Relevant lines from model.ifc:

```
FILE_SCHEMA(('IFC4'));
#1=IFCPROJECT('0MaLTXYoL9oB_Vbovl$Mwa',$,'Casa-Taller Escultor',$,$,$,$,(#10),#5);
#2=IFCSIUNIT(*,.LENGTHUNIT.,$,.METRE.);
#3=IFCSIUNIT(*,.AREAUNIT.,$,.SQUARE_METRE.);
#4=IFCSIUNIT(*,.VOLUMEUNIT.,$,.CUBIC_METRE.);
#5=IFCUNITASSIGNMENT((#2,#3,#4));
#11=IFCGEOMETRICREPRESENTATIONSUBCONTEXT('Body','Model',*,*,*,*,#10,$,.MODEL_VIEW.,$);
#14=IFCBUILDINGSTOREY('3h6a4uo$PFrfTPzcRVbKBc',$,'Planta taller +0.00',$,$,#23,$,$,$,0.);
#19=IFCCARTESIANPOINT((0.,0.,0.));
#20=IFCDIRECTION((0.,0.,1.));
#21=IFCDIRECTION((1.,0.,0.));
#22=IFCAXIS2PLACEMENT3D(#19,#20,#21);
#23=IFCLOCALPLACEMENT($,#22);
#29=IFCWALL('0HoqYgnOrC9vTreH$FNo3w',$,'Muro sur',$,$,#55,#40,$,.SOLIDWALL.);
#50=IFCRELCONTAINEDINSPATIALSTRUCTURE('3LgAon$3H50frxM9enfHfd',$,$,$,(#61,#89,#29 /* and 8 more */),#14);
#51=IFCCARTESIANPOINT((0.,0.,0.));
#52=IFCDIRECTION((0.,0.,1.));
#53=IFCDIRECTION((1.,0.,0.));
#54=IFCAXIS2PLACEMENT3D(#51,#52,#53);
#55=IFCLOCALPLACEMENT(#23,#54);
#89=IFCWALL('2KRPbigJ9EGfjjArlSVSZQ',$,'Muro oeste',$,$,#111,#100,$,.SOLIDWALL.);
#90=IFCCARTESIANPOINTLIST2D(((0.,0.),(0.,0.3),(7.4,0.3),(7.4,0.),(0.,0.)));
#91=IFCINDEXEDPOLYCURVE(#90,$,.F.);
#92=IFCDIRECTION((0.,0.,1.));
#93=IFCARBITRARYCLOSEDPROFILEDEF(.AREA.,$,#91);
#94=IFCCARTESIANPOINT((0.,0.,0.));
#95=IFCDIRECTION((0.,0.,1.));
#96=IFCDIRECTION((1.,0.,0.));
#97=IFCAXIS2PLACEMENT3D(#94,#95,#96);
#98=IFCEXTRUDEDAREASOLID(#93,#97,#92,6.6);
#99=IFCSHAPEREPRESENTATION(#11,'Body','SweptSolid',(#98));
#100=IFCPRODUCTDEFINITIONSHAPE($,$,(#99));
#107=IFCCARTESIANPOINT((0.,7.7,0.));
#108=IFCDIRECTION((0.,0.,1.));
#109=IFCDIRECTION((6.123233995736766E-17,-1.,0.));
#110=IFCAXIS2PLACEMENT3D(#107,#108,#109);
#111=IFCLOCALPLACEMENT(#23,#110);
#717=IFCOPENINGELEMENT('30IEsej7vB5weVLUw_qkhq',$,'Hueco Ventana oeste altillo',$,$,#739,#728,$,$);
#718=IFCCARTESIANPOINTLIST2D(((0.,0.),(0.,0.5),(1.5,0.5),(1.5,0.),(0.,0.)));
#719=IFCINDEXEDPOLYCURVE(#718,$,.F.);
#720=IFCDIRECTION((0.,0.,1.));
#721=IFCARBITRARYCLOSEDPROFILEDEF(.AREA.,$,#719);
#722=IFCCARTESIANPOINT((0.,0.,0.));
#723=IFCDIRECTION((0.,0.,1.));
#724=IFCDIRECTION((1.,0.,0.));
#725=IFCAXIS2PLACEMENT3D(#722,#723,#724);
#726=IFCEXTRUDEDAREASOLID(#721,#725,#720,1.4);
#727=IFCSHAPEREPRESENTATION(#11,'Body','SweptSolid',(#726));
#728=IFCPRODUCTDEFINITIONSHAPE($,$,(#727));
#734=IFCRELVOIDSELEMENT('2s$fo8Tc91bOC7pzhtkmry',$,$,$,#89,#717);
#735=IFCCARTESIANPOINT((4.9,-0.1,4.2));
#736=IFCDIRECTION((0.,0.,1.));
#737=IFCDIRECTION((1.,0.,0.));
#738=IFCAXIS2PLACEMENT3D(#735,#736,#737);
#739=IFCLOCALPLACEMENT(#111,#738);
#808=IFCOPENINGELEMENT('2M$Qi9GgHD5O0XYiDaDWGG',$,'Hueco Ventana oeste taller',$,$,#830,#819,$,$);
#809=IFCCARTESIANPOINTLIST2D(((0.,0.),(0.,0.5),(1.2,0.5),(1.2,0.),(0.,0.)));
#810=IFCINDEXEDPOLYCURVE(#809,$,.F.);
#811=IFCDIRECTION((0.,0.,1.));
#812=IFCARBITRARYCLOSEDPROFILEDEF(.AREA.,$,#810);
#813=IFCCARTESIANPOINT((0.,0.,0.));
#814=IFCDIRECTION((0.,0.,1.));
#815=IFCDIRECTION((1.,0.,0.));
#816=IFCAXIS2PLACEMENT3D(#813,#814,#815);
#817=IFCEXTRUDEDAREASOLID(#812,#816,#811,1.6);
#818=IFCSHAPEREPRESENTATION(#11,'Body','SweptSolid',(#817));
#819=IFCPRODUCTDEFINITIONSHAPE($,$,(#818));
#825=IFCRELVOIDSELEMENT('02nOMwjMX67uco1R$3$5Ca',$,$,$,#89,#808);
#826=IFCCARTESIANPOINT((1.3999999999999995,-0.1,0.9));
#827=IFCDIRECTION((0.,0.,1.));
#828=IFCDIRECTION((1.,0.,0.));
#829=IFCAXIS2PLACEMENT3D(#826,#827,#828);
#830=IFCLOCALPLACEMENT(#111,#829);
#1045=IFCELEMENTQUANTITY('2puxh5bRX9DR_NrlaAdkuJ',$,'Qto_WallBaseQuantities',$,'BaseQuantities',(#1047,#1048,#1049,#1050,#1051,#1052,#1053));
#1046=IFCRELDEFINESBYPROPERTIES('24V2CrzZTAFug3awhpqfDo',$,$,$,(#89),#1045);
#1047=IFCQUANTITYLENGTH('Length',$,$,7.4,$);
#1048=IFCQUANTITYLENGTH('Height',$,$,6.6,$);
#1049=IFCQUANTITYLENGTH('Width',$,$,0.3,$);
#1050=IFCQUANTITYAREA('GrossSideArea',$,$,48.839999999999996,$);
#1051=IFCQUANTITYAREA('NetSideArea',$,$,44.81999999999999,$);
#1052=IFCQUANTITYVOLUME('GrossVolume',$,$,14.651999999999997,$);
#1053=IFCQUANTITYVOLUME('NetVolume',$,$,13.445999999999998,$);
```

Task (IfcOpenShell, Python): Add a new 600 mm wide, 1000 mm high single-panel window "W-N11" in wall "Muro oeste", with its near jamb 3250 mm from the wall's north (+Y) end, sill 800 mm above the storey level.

```python
import numpy as np
import ifcopenshell
import ifcopenshell.api.feature
import ifcopenshell.api.geometry
import ifcopenshell.api.pset
import ifcopenshell.api.root
import ifcopenshell.api.spatial
import ifcopenshell.geom
import ifcopenshell.util.element
import ifcopenshell.util.placement
import ifcopenshell.util.representation
import ifcopenshell.util.shape
import ifcopenshell.util.unit

model = ifcopenshell.open("model.ifc")
unit_scale = ifcopenshell.util.unit.calculate_unit_scale(model)
area_scale = ifcopenshell.util.unit.calculate_unit_scale(model, "AREAUNIT")
volume_scale = ifcopenshell.util.unit.calculate_unit_scale(model, "VOLUMEUNIT")
settings = ifcopenshell.geom.settings()


def volume(element):
    """Net volume in cubic metres, openings subtracted."""
    shape = ifcopenshell.geom.create_shape(settings, element)
    return ifcopenshell.util.shape.get_volume(shape.geometry)


wall = model.by_id(89)
storey = ifcopenshell.util.element.get_container(wall, ifc_class="IfcBuildingStorey")
context = ifcopenshell.util.representation.get_context(model, "Model", "Body", "MODEL_VIEW")
before = volume(wall)

width, height, from_end, sill = 0.6, 1, 3.25, 0.8  # metres

# The wall runs along its own X axis, and the end named is its -X end.
wall_shape = ifcopenshell.geom.create_shape(settings, wall)
x, y, z = ifcopenshell.util.shape.get_vertices(wall_shape.geometry).T
start = x.min() + from_end
face, thickness = float(y.min()), float(y.max() - y.min())
wall_matrix = ifcopenshell.util.placement.get_local_placement(wall.ObjectPlacement)
level = ifcopenshell.util.placement.get_local_placement(storey.ObjectPlacement)[2, 3]


def in_wall(x, y):
    """Placement at x, y metres in the wall's axes, at sill height."""
    matrix = wall_matrix.copy()
    matrix[:, 3] = wall_matrix @ np.array([x / unit_scale, y / unit_scale, 0.0, 1.0])
    matrix[2, 3] = level + sill / unit_scale
    return matrix


# Opening: a box that overshoots both wall faces by 50 mm.
opening = ifcopenshell.api.root.create_entity(model, ifc_class="IfcOpeningElement", predefined_type="OPENING")
box = ifcopenshell.api.geometry.add_wall_representation(
    model, context=context, length=width, height=height, thickness=thickness + 0.1
)
ifcopenshell.api.geometry.assign_representation(model, product=opening, representation=box)
ifcopenshell.api.geometry.edit_object_placement(model, product=opening, matrix=in_wall(start, face - 0.05), is_si=False)
ifcopenshell.api.feature.add_feature(model, feature=opening, element=wall)

window = ifcopenshell.api.root.create_entity(model, ifc_class="IfcWindow", name="W-N11", predefined_type="WINDOW")
window.OverallWidth, window.OverallHeight = width / unit_scale, height / unit_scale
window.PartitioningType = "SINGLE_PANEL"
body = ifcopenshell.api.geometry.add_window_representation(
    model,
    context=context,
    overall_width=window.OverallWidth,
    overall_height=window.OverallHeight,
    partition_type="SINGLE_PANEL",
)
ifcopenshell.api.geometry.assign_representation(model, product=window, representation=body)
ifcopenshell.api.spatial.assign_container(model, products=[window], relating_structure=storey)
ifcopenshell.api.feature.add_filling(model, opening=opening, element=window)

# Centre the window in the wall's thickness.
ifcopenshell.api.geometry.edit_object_placement(model, product=window, matrix=in_wall(start, face), is_si=False)
window_shape = ifcopenshell.geom.create_shape(settings, window)
depth = ifcopenshell.util.shape.get_vertices(window_shape.geometry)[:, 1]
offset = face + thickness / 2 - (depth.min() + depth.max()) / 2
ifcopenshell.api.geometry.edit_object_placement(model, product=window, matrix=in_wall(start, offset), is_si=False)

after = volume(wall)

# Update the wall's stored quantities.
qto = model.by_id(ifcopenshell.util.element.get_pset(wall, "Qto_WallBaseQuantities", should_inherit=False)["id"])
ifcopenshell.api.pset.edit_qto(model, qto=qto, properties={
    "NetSideArea": after / thickness / area_scale,
    "NetVolume": after / volume_scale,
})

print(f"wall volume {before:.3f} -> {after:.3f} m3")

model.write("model_v2.ifc")
```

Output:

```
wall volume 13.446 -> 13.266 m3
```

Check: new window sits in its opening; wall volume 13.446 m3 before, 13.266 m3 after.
